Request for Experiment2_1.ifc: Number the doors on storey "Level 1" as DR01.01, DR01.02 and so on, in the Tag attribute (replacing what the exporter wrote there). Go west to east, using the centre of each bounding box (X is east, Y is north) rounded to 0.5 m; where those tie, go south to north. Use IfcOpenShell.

First a look at what the model holds.

```python
import ifcopenshell
import ifcopenshell.util.element
import ifcopenshell.util.placement

model = ifcopenshell.open("Experiment2_1.ifc")
print(model.schema)
storey = next(s for s in model.by_type("IfcBuildingStorey") if s.Name == "Level 1")
doors = [e for e in ifcopenshell.util.element.get_decomposition(storey) if e.is_a("IfcDoor")]
for e in sorted(doors, key=lambda e: e.id()):
    origin = ifcopenshell.util.placement.get_local_placement(e.ObjectPlacement)[:3, 3]
    print(e.id(), e.Tag, e.Name, origin.round(2) + 0.0, sep=" | ")
```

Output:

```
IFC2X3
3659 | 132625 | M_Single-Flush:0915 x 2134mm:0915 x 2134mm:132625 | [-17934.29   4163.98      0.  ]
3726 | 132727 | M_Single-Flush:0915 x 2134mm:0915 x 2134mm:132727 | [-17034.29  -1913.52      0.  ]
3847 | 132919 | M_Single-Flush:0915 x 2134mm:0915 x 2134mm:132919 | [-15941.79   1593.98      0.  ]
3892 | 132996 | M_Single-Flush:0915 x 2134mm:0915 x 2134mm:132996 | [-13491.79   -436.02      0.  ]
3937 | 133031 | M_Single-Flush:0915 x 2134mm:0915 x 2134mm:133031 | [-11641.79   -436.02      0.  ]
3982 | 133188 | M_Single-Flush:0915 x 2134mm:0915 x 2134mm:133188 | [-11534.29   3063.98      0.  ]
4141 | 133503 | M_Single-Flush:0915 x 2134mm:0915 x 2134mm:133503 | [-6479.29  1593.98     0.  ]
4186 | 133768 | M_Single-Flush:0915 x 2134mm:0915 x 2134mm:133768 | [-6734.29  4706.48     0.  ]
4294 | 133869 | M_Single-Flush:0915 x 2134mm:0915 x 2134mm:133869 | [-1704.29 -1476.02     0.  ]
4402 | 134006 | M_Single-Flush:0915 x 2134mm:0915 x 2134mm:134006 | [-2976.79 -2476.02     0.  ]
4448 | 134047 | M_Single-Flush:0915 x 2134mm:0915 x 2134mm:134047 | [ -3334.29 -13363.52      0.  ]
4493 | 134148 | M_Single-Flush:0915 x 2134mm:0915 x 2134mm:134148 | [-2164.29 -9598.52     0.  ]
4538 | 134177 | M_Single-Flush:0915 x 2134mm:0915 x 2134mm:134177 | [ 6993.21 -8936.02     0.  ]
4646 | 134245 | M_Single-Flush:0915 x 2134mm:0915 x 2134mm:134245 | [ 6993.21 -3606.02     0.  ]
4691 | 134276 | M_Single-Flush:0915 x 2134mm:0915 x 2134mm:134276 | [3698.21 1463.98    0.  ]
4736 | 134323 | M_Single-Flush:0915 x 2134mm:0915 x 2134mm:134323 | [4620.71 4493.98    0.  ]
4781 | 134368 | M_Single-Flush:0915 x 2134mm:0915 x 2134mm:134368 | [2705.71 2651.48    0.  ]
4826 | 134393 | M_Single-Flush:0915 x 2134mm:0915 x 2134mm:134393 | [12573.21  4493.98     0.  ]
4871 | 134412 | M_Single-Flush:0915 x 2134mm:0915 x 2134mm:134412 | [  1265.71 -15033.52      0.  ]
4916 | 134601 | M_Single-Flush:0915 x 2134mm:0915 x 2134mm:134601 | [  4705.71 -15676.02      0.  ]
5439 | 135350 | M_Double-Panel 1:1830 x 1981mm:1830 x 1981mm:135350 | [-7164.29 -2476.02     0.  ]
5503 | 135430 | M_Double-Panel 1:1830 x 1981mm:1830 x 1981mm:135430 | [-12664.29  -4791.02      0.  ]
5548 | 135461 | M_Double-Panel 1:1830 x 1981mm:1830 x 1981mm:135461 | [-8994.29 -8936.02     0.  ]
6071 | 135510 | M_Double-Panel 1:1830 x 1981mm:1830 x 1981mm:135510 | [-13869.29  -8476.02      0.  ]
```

```python
import ifcopenshell
import ifcopenshell.geom
import ifcopenshell.util.element
import ifcopenshell.util.shape

model = ifcopenshell.open("Experiment2_1.ifc")
settings = ifcopenshell.geom.settings()
settings.set("use-world-coords", True)


def centre(element):
    shape = ifcopenshell.geom.create_shape(settings, element)
    return ifcopenshell.util.shape.get_bbox_centroid(shape.geometry)


storey = next(s for s in model.by_type("IfcBuildingStorey") if s.Name == "Level 1")
doors = [e for e in ifcopenshell.util.element.get_decomposition(storey) if e.is_a("IfcDoor")]

# Insertion points can sit at a corner or the storey origin, so sort by the geometry (in metres).
centres = {e: centre(e) for e in doors}
doors.sort(key=lambda e: (round(centres[e][0] / 0.5), centres[e][1]))

for i, e in enumerate(doors, start=1):
    number = f"DR01.{i:02d}"
    e.Tag = number
    print(e.id(), number)

model.write("Experiment2_1_updated.ifc")
```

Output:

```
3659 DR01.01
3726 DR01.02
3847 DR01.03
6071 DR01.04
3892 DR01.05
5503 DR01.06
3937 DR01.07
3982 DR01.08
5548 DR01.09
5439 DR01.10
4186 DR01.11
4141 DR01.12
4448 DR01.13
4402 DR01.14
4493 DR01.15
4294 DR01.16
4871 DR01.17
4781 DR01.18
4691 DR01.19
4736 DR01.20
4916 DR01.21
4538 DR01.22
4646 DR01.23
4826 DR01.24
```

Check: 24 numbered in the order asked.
